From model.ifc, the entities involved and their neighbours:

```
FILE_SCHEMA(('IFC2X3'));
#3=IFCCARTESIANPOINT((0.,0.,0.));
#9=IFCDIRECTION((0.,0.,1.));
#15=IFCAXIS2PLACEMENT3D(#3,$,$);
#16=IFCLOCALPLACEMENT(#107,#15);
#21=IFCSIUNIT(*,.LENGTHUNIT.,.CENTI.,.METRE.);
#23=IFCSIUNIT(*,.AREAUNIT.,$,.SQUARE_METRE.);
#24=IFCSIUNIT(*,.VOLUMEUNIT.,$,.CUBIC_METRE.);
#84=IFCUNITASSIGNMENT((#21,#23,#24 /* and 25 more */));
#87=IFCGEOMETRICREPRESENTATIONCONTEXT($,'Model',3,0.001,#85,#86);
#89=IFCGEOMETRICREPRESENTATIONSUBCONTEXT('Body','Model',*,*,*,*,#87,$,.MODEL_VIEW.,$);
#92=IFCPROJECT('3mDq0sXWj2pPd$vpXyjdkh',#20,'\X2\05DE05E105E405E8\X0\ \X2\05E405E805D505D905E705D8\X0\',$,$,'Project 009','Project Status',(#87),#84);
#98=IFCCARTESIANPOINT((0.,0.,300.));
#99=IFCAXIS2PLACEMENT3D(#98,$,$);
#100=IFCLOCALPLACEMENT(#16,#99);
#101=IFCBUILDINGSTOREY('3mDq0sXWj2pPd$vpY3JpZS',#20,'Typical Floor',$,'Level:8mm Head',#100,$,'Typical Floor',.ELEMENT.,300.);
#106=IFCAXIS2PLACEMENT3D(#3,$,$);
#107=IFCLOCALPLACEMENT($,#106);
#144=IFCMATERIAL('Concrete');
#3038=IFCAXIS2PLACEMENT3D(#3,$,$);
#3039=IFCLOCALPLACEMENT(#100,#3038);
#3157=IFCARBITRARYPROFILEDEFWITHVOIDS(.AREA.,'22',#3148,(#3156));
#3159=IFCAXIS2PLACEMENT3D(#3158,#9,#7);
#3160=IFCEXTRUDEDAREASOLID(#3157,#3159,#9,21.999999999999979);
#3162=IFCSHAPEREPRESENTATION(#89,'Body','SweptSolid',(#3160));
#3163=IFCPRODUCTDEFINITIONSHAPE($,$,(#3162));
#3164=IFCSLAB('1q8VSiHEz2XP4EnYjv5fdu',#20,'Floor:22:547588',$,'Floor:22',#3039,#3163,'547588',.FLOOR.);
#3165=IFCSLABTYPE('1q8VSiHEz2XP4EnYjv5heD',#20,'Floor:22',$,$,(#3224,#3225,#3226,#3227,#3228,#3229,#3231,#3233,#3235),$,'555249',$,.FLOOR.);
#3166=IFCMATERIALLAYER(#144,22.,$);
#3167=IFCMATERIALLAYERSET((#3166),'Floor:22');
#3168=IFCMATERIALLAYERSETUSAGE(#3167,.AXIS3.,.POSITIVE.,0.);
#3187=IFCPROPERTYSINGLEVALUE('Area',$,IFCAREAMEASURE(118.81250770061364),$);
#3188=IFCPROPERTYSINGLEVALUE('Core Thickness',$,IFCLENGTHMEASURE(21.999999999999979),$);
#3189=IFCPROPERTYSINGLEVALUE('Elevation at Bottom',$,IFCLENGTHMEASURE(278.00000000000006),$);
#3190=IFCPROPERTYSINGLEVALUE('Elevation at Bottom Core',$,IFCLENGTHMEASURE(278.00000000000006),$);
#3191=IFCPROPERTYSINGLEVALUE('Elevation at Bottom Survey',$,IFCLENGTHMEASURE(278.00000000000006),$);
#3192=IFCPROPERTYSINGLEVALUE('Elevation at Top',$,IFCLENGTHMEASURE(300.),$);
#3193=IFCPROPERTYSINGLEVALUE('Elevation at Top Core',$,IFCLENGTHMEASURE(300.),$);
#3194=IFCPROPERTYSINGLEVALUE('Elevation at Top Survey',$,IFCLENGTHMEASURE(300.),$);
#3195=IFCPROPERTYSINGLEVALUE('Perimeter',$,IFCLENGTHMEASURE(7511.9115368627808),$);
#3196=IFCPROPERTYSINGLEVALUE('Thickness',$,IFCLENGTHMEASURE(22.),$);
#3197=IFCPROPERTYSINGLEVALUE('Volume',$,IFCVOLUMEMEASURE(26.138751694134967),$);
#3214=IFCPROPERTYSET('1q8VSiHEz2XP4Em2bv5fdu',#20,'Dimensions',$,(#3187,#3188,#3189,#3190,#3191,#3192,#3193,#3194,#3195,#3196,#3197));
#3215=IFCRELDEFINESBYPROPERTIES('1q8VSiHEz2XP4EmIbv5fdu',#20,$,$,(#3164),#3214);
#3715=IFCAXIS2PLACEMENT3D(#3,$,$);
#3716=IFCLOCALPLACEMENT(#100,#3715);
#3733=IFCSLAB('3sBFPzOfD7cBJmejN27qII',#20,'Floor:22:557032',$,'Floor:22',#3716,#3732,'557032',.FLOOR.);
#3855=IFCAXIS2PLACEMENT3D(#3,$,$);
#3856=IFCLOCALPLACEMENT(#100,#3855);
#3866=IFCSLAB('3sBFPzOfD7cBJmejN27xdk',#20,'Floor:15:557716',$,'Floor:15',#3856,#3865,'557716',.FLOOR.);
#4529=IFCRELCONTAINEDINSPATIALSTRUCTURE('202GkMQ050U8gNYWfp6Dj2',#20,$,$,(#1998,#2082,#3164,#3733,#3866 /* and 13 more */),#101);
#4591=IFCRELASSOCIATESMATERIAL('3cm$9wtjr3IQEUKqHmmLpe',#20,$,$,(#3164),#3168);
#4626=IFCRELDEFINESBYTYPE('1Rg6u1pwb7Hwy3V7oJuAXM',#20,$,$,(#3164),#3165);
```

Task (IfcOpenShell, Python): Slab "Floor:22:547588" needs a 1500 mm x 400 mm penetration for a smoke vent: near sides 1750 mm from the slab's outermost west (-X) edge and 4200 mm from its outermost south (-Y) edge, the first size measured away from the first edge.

```python
import numpy as np
import ifcopenshell
import ifcopenshell.api.feature
import ifcopenshell.api.geometry
import ifcopenshell.api.pset
import ifcopenshell.api.root
import ifcopenshell.geom
import ifcopenshell.util.element
import ifcopenshell.util.placement
import ifcopenshell.util.representation
import ifcopenshell.util.shape
import ifcopenshell.util.unit

model = ifcopenshell.open("model.ifc")
unit_scale = ifcopenshell.util.unit.calculate_unit_scale(model)
area_scale = ifcopenshell.util.unit.calculate_unit_scale(model, "AREAUNIT")
volume_scale = ifcopenshell.util.unit.calculate_unit_scale(model, "VOLUMEUNIT")
settings = ifcopenshell.geom.settings()


def volume(element):
    """Net volume in cubic metres, openings subtracted."""
    shape = ifcopenshell.geom.create_shape(settings, element)
    return ifcopenshell.util.shape.get_volume(shape.geometry)


slab = model.by_id(3164)
before = volume(slab)

# Extent in the slab's own axes, in metres. The edges named are its -X and -Y sides.
slab_shape = ifcopenshell.geom.create_shape(settings, slab)
vertices = ifcopenshell.util.shape.get_vertices(slab_shape.geometry)
x_min, y_min, bottom = vertices.min(axis=0)
top = vertices[:, 2].max()

opening = ifcopenshell.api.root.create_entity(model, ifc_class="IfcOpeningElement", name="Smoke vent opening")
context = ifcopenshell.util.representation.get_context(model, "Model", "Body", "MODEL_VIEW")
width, depth = 1.5, 0.4
outline = [(0.0, 0.0), (width, 0.0), (width, depth), (0.0, depth), (0.0, 0.0)]
# Overshoot both faces by 50 mm so the cut is clean.
shape = ifcopenshell.api.geometry.add_slab_representation(
    model, context=context, depth=top - bottom + 0.1, polyline=outline
)
ifcopenshell.api.geometry.assign_representation(model, product=opening, representation=shape)

matrix = ifcopenshell.util.placement.get_local_placement(slab.ObjectPlacement)
matrix[:, 3] = matrix @ np.append(np.array([x_min + 1.75, y_min + 4.2, bottom - 0.05]) / unit_scale, 1.0)
ifcopenshell.api.geometry.edit_object_placement(model, product=opening, matrix=matrix, is_si=False)
ifcopenshell.api.feature.add_feature(model, feature=opening, element=slab)

after = volume(slab)

# Update the slab's stored quantities.
pset = model.by_id(ifcopenshell.util.element.get_pset(slab, "Dimensions", should_inherit=False)["id"])
ifcopenshell.api.pset.edit_pset(model, pset=pset, properties={
    "Area": model.create_entity("IfcAreaMeasure", after / (top - bottom) / area_scale),
    "Volume": model.create_entity("IfcVolumeMeasure", after / volume_scale),
})

print(f"slab volume {before:.3f} -> {after:.3f} m3")

model.write("model_rev.ifc")
```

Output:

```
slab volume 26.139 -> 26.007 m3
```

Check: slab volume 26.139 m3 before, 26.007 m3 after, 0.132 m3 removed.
